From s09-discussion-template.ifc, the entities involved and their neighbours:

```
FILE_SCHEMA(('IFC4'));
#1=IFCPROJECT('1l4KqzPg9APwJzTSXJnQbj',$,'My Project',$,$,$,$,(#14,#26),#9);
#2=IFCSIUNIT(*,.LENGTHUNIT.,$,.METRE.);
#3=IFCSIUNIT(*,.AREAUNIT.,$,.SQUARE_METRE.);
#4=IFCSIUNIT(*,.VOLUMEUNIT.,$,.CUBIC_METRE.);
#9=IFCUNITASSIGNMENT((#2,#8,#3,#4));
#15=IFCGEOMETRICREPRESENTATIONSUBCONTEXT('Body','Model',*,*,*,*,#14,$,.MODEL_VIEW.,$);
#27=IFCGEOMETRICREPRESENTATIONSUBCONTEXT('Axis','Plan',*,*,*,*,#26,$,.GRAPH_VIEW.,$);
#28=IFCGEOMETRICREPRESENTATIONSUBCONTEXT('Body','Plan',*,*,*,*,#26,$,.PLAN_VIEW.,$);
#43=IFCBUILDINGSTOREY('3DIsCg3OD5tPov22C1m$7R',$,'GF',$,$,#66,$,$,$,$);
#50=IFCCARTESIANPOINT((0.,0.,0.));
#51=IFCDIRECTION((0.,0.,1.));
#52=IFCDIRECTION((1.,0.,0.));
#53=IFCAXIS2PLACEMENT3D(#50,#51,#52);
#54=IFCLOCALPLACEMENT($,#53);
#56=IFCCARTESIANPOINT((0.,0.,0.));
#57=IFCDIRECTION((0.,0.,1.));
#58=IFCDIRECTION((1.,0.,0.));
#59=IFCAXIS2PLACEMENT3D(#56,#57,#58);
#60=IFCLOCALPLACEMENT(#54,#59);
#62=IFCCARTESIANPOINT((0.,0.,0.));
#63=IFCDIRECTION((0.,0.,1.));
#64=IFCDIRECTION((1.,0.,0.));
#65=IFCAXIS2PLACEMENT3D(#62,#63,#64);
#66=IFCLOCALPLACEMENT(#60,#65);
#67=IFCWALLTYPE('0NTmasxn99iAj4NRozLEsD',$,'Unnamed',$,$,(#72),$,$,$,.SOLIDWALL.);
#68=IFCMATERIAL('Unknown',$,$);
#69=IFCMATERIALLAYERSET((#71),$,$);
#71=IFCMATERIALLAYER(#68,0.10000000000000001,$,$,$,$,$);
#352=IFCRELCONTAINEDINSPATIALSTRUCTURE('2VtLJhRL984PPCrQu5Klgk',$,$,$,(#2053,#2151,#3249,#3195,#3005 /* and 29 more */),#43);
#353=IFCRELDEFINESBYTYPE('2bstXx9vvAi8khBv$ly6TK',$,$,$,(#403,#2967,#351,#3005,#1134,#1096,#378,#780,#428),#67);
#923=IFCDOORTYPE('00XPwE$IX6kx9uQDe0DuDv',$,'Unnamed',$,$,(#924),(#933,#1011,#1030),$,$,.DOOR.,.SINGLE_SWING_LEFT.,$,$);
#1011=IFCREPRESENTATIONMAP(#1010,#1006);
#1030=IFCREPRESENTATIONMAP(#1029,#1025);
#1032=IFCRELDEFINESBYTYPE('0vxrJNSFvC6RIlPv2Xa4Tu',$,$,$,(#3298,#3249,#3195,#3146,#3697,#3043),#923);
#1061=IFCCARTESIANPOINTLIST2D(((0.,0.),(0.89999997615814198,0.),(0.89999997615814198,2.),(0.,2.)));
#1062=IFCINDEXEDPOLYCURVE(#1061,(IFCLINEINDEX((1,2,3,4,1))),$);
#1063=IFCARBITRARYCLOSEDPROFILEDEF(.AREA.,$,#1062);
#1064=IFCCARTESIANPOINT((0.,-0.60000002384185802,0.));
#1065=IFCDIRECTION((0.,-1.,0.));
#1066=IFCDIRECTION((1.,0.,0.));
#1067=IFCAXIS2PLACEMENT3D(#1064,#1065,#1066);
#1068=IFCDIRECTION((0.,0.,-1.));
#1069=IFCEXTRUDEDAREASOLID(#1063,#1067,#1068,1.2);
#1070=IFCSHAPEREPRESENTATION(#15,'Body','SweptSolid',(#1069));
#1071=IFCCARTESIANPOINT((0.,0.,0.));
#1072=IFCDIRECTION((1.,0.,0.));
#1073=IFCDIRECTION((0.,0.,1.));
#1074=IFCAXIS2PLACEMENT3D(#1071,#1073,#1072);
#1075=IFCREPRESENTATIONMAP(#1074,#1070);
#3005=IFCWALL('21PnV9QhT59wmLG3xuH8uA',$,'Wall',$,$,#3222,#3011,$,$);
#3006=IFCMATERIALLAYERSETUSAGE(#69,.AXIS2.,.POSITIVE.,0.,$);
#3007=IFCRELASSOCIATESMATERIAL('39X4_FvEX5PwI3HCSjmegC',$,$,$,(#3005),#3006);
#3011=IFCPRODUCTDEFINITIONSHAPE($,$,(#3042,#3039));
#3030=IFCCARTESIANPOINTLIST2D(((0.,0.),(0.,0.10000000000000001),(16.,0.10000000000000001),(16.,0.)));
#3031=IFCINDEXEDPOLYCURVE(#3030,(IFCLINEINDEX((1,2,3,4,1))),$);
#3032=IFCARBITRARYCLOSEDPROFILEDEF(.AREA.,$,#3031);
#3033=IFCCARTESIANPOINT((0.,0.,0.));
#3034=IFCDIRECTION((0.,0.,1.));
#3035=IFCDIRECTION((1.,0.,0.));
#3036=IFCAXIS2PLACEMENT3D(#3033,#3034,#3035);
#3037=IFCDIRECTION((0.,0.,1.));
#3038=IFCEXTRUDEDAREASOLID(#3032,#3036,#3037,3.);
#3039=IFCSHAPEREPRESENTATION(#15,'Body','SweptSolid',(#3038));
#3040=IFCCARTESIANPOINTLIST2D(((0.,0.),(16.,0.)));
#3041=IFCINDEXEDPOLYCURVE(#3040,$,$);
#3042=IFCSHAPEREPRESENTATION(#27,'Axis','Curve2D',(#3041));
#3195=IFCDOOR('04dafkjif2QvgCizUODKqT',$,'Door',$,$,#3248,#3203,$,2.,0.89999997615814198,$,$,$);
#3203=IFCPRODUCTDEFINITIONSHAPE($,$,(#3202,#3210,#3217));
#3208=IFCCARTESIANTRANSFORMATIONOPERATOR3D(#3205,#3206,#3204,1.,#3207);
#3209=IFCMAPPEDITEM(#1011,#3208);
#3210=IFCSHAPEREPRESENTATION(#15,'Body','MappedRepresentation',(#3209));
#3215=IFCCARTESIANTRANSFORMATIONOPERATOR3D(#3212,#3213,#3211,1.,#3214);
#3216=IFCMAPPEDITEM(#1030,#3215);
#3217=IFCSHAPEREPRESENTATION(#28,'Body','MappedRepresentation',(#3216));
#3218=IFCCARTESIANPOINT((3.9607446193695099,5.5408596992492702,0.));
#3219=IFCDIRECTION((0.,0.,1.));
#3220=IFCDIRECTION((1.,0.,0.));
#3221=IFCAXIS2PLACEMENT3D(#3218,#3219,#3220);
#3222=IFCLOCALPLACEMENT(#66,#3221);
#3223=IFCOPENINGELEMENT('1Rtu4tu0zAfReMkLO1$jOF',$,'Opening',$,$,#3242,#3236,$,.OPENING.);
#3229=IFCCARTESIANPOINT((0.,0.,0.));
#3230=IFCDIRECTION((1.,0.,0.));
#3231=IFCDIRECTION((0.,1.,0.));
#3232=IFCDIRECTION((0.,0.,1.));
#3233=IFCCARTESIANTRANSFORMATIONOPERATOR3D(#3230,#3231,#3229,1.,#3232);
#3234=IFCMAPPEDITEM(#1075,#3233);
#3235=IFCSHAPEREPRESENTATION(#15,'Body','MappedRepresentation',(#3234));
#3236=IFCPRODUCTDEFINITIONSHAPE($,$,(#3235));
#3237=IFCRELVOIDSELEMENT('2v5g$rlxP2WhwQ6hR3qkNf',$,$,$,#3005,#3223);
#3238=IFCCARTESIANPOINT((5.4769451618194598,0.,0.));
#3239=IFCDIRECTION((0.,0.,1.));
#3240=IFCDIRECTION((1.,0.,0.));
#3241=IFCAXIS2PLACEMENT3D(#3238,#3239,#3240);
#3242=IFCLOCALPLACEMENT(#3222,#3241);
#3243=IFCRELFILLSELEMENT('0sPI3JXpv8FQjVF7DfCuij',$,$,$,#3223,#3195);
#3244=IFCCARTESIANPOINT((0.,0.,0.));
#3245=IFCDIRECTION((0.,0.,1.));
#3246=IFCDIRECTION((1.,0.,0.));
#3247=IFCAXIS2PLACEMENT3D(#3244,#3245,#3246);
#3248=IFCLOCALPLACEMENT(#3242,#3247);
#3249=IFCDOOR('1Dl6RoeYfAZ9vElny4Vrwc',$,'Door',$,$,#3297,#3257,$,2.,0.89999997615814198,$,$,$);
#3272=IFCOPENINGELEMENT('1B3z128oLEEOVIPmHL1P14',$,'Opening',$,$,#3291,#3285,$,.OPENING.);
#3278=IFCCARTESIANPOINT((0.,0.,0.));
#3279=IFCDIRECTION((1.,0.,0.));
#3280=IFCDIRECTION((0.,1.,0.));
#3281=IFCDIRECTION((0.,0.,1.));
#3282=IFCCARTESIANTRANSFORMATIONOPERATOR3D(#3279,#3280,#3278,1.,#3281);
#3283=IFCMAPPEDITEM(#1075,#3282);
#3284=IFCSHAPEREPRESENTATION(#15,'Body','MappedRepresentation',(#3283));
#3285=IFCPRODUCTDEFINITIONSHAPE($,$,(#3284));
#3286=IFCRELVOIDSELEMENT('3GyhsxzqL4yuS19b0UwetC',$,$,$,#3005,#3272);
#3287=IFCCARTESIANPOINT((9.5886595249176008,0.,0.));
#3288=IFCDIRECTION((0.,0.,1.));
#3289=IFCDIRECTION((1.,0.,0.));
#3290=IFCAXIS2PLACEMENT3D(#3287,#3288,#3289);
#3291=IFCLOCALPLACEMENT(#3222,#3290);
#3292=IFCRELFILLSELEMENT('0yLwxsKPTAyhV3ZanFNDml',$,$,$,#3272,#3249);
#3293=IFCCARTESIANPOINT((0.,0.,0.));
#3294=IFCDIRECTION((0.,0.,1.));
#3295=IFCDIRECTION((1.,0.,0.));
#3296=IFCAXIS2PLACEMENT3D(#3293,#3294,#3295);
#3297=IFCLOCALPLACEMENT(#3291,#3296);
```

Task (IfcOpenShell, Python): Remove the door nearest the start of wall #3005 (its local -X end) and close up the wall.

```python
import ifcopenshell
import ifcopenshell.api.feature
import ifcopenshell.api.root
import ifcopenshell.geom
import ifcopenshell.util.shape

model = ifcopenshell.open("s09-discussion-template.ifc")
settings = ifcopenshell.geom.settings()


def volume(element):
    """Net volume in cubic metres, openings subtracted."""
    shape = ifcopenshell.geom.create_shape(settings, element)
    return ifcopenshell.util.shape.get_volume(shape.geometry)


door = model.by_guid("04dafkjif2QvgCizUODKqT")
opening = door.FillsVoids[0].RelatingOpeningElement
wall = opening.VoidsElements[0].RelatingBuildingElement
before = volume(wall)

ifcopenshell.api.root.remove_product(model, product=door)
ifcopenshell.api.feature.remove_feature(model, feature=opening)

after = volume(wall)

print(f"wall volume {before:.3f} -> {after:.3f} m3")

model.write("s09-discussion-template_v2.ifc")
```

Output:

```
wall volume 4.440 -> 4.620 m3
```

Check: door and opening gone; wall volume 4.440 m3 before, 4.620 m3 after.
